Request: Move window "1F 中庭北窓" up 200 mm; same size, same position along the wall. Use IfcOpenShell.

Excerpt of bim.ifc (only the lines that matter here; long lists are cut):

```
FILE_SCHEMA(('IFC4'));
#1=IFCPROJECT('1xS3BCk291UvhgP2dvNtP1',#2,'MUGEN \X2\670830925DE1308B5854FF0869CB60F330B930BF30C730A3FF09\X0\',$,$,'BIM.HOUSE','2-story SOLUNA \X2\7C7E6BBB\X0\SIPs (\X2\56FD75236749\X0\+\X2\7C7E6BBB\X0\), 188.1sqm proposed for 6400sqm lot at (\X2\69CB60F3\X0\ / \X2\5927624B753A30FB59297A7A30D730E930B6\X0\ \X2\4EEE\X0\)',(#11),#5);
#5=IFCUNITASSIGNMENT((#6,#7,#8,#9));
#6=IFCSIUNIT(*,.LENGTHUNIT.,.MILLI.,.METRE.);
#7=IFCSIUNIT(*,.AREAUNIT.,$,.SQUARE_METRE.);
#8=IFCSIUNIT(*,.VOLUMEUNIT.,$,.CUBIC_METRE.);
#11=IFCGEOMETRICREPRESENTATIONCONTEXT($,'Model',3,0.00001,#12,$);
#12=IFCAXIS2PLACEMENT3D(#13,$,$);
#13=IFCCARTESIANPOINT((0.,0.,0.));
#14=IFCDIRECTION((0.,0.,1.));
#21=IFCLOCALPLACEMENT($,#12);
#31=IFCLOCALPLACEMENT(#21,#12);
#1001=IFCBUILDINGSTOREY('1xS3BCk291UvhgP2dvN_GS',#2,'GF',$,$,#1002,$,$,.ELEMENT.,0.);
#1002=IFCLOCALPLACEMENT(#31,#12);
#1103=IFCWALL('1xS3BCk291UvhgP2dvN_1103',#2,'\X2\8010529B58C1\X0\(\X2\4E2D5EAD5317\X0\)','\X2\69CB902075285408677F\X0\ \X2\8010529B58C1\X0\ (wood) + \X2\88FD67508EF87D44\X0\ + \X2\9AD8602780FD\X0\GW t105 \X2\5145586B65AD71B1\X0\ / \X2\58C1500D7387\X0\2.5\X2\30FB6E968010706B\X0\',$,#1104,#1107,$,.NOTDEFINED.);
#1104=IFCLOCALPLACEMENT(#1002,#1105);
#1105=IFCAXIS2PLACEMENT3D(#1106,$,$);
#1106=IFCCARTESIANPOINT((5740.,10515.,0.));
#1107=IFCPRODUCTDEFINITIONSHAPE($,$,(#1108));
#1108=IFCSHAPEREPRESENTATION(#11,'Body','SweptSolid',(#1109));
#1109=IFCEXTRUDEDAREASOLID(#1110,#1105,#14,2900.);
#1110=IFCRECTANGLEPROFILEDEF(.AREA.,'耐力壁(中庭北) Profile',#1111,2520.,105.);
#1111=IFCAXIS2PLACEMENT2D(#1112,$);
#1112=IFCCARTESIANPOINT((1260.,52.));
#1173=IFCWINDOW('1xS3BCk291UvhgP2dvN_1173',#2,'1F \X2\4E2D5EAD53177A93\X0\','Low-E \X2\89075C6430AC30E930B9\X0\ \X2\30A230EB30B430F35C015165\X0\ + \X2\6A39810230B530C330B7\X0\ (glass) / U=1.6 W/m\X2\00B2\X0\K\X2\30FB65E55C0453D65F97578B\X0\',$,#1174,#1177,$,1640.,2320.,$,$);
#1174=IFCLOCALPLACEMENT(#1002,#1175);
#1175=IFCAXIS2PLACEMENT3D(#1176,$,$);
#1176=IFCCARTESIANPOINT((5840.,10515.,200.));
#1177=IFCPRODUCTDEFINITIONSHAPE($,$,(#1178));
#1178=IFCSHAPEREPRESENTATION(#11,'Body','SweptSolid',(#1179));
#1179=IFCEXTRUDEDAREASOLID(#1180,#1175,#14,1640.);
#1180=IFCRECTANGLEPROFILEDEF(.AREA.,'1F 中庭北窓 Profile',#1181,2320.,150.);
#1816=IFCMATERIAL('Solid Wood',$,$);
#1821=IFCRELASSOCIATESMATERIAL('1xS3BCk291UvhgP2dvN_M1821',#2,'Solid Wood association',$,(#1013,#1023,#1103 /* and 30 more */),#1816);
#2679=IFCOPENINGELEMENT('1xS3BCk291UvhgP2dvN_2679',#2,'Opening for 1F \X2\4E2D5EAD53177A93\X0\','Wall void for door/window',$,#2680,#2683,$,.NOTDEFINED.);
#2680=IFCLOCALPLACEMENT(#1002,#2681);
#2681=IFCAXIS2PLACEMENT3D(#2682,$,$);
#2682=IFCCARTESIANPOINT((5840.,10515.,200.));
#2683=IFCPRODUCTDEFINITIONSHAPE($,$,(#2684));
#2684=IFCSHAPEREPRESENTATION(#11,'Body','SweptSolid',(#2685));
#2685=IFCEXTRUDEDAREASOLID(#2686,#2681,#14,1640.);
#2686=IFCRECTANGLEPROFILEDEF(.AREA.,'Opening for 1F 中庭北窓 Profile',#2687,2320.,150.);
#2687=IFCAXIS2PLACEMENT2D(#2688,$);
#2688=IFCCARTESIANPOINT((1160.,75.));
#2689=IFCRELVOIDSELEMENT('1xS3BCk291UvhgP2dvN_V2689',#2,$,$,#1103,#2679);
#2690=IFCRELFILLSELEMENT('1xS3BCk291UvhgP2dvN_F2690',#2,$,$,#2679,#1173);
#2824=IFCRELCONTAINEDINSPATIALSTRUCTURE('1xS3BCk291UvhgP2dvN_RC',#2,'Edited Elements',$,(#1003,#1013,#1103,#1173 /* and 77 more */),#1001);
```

```python
import numpy as np
import ifcopenshell
import ifcopenshell.api.geometry
import ifcopenshell.util.placement
import ifcopenshell.util.unit

model = ifcopenshell.open("bim.ifc")
unit_scale = ifcopenshell.util.unit.calculate_unit_scale(model)

window = model.by_guid("1xS3BCk291UvhgP2dvN_1173")
opening = window.FillsVoids[0].RelatingOpeningElement
dz = 0.2 / unit_scale

shift = np.array([0.0, 0.0, dz])
# The window is not placed relative to its opening, so move both.
for product in (opening, window):
    matrix = ifcopenshell.util.placement.get_local_placement(product.ObjectPlacement)
    matrix[:3, 3] += shift
    ifcopenshell.api.geometry.edit_object_placement(model, product=product, matrix=matrix, is_si=False)

print(f"moved by {dz * unit_scale:+.3f} m")

model.write("bim_edited.ifc")
```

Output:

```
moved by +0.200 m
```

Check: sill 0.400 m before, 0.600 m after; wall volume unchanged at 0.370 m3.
